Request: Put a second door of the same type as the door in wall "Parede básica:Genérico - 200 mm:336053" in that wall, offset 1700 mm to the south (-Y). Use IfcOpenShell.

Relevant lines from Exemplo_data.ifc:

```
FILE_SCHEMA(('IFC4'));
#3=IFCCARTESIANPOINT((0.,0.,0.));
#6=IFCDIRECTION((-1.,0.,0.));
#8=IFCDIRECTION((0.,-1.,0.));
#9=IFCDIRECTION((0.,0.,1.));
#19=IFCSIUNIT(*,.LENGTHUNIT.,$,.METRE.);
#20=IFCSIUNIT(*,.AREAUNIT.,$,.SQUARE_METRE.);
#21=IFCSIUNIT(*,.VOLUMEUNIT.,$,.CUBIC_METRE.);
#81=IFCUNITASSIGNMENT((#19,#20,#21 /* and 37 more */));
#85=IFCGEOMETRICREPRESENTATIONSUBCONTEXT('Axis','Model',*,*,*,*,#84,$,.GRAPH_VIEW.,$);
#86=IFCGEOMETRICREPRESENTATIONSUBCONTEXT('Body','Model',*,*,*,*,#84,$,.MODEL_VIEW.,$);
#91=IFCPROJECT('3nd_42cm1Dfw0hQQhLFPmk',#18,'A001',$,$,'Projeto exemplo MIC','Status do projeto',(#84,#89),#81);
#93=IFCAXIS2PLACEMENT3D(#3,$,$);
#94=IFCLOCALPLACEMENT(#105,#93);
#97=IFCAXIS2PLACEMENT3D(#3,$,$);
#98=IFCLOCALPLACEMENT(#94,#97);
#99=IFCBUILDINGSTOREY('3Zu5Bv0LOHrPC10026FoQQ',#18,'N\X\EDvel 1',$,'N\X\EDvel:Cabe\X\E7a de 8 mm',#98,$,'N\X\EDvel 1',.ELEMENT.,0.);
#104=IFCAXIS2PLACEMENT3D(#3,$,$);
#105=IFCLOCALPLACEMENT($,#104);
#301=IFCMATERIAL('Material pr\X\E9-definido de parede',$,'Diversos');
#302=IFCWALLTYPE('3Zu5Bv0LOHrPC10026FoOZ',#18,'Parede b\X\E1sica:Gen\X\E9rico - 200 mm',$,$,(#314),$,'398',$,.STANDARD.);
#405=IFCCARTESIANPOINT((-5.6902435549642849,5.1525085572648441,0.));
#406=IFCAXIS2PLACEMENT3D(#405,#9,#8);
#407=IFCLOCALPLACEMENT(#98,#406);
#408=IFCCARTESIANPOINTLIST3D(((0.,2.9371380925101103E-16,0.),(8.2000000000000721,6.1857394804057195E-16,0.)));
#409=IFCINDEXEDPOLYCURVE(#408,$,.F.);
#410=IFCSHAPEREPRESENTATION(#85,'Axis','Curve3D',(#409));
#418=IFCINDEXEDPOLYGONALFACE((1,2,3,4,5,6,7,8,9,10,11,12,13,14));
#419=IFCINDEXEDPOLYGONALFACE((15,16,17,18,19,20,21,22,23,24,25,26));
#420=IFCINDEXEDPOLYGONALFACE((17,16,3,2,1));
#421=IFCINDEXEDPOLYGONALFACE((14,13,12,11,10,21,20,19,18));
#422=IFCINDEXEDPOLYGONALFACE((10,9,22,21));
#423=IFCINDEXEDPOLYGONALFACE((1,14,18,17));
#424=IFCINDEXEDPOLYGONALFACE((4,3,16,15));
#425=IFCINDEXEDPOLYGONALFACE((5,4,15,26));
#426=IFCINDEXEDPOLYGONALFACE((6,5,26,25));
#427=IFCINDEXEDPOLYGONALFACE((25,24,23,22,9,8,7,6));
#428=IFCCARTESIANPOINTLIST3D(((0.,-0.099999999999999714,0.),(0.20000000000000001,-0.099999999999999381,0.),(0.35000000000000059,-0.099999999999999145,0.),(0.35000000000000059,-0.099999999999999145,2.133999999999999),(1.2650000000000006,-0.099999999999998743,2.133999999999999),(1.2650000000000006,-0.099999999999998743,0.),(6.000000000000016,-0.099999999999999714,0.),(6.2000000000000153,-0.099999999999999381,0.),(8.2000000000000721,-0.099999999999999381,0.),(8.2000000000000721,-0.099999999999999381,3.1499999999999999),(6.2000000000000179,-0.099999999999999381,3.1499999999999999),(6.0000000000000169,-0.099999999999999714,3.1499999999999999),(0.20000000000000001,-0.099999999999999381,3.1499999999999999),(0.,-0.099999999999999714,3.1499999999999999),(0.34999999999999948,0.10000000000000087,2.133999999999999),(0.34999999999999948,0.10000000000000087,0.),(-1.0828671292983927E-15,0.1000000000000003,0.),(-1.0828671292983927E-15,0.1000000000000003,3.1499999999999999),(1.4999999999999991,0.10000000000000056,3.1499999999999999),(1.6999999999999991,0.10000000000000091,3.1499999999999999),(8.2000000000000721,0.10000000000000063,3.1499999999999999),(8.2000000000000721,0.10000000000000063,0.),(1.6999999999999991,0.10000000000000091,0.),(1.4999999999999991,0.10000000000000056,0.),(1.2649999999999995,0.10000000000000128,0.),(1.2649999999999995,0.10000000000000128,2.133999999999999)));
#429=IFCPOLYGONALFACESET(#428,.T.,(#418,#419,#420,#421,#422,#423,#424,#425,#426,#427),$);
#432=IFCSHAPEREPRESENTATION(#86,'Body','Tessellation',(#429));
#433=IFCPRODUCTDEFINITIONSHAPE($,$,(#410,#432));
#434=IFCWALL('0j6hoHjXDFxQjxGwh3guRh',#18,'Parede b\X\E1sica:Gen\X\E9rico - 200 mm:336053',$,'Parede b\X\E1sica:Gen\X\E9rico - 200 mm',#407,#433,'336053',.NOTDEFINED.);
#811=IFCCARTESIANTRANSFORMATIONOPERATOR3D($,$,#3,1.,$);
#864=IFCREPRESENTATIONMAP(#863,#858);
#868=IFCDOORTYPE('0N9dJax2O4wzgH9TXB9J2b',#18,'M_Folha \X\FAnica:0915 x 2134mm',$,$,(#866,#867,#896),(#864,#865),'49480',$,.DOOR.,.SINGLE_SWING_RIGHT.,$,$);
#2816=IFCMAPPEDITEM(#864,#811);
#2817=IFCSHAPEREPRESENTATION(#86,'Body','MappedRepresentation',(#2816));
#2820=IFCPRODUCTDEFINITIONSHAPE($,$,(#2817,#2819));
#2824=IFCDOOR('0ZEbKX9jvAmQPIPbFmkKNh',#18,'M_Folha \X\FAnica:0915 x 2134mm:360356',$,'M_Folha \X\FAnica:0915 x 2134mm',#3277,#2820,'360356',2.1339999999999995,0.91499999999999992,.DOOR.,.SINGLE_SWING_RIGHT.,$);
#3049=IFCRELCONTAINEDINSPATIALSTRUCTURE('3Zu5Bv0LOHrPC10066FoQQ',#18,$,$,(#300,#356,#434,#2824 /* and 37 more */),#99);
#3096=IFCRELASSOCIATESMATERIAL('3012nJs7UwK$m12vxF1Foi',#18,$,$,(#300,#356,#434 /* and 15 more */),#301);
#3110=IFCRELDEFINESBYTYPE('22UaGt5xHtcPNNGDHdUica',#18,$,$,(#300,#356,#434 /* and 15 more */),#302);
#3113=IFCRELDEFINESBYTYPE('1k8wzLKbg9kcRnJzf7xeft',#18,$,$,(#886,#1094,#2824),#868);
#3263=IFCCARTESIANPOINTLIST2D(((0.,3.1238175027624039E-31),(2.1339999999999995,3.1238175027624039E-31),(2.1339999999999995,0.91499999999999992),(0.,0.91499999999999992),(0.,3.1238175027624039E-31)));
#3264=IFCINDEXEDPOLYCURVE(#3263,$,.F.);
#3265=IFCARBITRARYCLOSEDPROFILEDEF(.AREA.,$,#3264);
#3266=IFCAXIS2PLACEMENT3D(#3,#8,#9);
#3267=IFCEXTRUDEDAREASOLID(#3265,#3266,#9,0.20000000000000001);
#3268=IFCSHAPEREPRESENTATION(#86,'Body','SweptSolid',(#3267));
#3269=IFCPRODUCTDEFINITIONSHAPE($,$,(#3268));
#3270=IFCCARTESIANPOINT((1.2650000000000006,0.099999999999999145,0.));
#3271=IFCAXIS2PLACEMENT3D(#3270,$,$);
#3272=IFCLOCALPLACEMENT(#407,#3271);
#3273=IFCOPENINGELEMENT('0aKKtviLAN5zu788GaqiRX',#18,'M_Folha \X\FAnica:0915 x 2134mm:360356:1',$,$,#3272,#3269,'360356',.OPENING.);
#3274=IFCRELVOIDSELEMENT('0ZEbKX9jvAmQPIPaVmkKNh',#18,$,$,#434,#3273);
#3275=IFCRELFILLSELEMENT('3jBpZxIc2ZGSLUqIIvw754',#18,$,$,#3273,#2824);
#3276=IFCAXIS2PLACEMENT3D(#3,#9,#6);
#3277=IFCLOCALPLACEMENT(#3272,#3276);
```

```python
import ifcopenshell
import ifcopenshell.api.feature
import ifcopenshell.api.geometry
import ifcopenshell.api.root
import ifcopenshell.geom
import ifcopenshell.util.element
import ifcopenshell.util.placement
import ifcopenshell.util.shape

model = ifcopenshell.open("Exemplo_data.ifc")
settings = ifcopenshell.geom.settings()


def volume(element):
    """Net volume in cubic metres, openings subtracted."""
    shape = ifcopenshell.geom.create_shape(settings, element)
    return ifcopenshell.util.shape.get_volume(shape.geometry)


def reuse_history(source, copy):
    """copy_class also copies each property set's owner history, people and application; keep the originals."""
    for rel in copy.IsDefinedBy:
        if rel.is_a("IfcRelDefinesByProperties") and (history := rel.RelatingPropertyDefinition.OwnerHistory):
            rel.RelatingPropertyDefinition.OwnerHistory = source.OwnerHistory
            ifcopenshell.util.element.remove_deep2(model, history)


door = model.by_id(2824)
opening = door.FillsVoids[0].RelatingOpeningElement
wall = opening.VoidsElements[0].RelatingBuildingElement
before = volume(wall)
shift = ifcopenshell.util.placement.get_local_placement(wall.ObjectPlacement)[:3, 0] * 1.7

# copy_class copies the void relationship, type, container and properties, but no geometry.
new_opening = ifcopenshell.api.root.copy_class(model, product=opening)
new_opening.Representation = ifcopenshell.util.element.copy_deep(
    model, opening.Representation, exclude=["IfcGeometricRepresentationContext", "IfcRepresentationMap"]
)
new_opening.Name = "M_Folha única:0915 x 2134mm"
new_opening.Tag = None
new_door = ifcopenshell.api.root.copy_class(model, product=door)
new_door.Representation = ifcopenshell.util.element.copy_deep(
    model, door.Representation, exclude=["IfcGeometricRepresentationContext", "IfcRepresentationMap"]
)
new_door.Name = "M_Folha única:0915 x 2134mm"
new_door.Tag = None
reuse_history(door, new_door)
ifcopenshell.api.feature.add_filling(model, opening=new_opening, element=new_door)

for old, new in ((opening, new_opening), (door, new_door)):
    matrix = ifcopenshell.util.placement.get_local_placement(old.ObjectPlacement)
    matrix[:3, 3] += shift
    ifcopenshell.api.geometry.edit_object_placement(model, product=new, matrix=matrix, is_si=False)

after = volume(wall)

print(f"wall volume {before:.3f} -> {after:.3f} m3")

model.write("Exemplo_data-out.ifc")
```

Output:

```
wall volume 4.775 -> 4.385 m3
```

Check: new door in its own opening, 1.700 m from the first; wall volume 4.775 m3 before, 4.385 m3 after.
